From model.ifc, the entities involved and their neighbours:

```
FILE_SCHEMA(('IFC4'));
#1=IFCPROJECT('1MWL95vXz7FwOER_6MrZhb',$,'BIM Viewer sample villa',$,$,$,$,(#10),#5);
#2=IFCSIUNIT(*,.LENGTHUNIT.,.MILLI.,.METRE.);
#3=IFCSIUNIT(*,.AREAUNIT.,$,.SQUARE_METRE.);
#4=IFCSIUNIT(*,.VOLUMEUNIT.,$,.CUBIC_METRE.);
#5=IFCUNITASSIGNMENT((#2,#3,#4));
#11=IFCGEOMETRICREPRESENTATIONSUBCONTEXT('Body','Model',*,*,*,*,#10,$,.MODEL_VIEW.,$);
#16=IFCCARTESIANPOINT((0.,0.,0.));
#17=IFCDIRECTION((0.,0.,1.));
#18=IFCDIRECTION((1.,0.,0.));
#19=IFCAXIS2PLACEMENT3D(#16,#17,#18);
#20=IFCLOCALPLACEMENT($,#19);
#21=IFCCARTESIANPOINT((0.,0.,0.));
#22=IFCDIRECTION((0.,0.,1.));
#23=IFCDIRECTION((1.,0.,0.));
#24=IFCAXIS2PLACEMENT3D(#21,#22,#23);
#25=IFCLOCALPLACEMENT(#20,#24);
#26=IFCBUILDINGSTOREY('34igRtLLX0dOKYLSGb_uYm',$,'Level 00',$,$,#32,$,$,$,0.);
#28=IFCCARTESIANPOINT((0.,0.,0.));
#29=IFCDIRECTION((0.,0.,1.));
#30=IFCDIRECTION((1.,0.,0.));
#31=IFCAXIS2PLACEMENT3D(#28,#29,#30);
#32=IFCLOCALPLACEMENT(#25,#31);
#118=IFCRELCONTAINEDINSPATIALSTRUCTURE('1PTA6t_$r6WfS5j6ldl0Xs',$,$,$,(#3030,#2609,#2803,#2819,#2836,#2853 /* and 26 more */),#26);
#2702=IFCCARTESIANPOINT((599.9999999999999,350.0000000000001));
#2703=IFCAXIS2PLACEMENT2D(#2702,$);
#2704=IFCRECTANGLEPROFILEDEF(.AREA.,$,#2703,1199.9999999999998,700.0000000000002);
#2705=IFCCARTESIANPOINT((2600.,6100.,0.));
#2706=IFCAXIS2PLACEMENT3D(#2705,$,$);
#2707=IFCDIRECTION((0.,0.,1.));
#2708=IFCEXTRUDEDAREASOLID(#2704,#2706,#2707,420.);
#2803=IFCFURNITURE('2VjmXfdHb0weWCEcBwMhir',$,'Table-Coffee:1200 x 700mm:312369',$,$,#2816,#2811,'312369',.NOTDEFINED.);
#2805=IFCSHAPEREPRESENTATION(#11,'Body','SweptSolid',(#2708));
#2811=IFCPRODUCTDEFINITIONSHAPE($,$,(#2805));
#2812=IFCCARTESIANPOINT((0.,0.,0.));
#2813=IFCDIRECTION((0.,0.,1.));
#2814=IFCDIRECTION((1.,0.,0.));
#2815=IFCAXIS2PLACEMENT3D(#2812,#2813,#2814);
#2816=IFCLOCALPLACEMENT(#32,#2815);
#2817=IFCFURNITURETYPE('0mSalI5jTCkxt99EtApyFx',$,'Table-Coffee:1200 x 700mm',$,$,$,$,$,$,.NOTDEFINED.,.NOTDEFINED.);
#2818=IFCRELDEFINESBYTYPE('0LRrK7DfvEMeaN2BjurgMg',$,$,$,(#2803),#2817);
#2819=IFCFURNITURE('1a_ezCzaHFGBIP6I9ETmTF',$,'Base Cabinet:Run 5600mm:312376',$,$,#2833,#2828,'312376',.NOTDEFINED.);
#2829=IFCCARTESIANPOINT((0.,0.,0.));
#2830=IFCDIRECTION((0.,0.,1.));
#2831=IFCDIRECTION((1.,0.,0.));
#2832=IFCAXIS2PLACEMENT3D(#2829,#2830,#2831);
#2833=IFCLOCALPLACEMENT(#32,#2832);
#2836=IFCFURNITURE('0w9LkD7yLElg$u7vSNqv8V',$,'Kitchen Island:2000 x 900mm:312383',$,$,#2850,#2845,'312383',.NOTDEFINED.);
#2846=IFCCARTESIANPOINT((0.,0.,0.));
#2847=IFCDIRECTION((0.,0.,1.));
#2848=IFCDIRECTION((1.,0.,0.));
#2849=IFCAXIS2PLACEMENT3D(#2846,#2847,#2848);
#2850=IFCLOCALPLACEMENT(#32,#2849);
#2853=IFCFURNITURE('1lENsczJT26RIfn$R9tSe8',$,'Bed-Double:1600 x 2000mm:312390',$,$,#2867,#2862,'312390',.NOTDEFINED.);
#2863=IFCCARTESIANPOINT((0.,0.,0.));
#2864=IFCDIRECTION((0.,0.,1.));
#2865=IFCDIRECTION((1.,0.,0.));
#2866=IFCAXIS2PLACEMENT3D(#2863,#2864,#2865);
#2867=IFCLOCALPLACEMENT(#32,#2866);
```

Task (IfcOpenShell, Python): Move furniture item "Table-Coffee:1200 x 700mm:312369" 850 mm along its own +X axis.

```python
import ifcopenshell
import ifcopenshell.api.geometry
import ifcopenshell.util.placement
import ifcopenshell.util.unit

model = ifcopenshell.open("model.ifc")
unit_scale = ifcopenshell.util.unit.calculate_unit_scale(model)

item = model.by_guid("2VjmXfdHb0weWCEcBwMhir")
matrix = ifcopenshell.util.placement.get_local_placement(item.ObjectPlacement)
matrix[:3, 3] += matrix[:3, 0] * 0.85 / unit_scale
ifcopenshell.api.geometry.edit_object_placement(model, product=item, matrix=matrix, is_si=False)

print(ifcopenshell.util.placement.get_local_placement(item.ObjectPlacement).round(3) + 0.0)

model.write("model_edited.ifc")
```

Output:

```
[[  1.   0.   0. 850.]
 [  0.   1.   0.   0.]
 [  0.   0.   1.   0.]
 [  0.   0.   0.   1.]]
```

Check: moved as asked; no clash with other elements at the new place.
